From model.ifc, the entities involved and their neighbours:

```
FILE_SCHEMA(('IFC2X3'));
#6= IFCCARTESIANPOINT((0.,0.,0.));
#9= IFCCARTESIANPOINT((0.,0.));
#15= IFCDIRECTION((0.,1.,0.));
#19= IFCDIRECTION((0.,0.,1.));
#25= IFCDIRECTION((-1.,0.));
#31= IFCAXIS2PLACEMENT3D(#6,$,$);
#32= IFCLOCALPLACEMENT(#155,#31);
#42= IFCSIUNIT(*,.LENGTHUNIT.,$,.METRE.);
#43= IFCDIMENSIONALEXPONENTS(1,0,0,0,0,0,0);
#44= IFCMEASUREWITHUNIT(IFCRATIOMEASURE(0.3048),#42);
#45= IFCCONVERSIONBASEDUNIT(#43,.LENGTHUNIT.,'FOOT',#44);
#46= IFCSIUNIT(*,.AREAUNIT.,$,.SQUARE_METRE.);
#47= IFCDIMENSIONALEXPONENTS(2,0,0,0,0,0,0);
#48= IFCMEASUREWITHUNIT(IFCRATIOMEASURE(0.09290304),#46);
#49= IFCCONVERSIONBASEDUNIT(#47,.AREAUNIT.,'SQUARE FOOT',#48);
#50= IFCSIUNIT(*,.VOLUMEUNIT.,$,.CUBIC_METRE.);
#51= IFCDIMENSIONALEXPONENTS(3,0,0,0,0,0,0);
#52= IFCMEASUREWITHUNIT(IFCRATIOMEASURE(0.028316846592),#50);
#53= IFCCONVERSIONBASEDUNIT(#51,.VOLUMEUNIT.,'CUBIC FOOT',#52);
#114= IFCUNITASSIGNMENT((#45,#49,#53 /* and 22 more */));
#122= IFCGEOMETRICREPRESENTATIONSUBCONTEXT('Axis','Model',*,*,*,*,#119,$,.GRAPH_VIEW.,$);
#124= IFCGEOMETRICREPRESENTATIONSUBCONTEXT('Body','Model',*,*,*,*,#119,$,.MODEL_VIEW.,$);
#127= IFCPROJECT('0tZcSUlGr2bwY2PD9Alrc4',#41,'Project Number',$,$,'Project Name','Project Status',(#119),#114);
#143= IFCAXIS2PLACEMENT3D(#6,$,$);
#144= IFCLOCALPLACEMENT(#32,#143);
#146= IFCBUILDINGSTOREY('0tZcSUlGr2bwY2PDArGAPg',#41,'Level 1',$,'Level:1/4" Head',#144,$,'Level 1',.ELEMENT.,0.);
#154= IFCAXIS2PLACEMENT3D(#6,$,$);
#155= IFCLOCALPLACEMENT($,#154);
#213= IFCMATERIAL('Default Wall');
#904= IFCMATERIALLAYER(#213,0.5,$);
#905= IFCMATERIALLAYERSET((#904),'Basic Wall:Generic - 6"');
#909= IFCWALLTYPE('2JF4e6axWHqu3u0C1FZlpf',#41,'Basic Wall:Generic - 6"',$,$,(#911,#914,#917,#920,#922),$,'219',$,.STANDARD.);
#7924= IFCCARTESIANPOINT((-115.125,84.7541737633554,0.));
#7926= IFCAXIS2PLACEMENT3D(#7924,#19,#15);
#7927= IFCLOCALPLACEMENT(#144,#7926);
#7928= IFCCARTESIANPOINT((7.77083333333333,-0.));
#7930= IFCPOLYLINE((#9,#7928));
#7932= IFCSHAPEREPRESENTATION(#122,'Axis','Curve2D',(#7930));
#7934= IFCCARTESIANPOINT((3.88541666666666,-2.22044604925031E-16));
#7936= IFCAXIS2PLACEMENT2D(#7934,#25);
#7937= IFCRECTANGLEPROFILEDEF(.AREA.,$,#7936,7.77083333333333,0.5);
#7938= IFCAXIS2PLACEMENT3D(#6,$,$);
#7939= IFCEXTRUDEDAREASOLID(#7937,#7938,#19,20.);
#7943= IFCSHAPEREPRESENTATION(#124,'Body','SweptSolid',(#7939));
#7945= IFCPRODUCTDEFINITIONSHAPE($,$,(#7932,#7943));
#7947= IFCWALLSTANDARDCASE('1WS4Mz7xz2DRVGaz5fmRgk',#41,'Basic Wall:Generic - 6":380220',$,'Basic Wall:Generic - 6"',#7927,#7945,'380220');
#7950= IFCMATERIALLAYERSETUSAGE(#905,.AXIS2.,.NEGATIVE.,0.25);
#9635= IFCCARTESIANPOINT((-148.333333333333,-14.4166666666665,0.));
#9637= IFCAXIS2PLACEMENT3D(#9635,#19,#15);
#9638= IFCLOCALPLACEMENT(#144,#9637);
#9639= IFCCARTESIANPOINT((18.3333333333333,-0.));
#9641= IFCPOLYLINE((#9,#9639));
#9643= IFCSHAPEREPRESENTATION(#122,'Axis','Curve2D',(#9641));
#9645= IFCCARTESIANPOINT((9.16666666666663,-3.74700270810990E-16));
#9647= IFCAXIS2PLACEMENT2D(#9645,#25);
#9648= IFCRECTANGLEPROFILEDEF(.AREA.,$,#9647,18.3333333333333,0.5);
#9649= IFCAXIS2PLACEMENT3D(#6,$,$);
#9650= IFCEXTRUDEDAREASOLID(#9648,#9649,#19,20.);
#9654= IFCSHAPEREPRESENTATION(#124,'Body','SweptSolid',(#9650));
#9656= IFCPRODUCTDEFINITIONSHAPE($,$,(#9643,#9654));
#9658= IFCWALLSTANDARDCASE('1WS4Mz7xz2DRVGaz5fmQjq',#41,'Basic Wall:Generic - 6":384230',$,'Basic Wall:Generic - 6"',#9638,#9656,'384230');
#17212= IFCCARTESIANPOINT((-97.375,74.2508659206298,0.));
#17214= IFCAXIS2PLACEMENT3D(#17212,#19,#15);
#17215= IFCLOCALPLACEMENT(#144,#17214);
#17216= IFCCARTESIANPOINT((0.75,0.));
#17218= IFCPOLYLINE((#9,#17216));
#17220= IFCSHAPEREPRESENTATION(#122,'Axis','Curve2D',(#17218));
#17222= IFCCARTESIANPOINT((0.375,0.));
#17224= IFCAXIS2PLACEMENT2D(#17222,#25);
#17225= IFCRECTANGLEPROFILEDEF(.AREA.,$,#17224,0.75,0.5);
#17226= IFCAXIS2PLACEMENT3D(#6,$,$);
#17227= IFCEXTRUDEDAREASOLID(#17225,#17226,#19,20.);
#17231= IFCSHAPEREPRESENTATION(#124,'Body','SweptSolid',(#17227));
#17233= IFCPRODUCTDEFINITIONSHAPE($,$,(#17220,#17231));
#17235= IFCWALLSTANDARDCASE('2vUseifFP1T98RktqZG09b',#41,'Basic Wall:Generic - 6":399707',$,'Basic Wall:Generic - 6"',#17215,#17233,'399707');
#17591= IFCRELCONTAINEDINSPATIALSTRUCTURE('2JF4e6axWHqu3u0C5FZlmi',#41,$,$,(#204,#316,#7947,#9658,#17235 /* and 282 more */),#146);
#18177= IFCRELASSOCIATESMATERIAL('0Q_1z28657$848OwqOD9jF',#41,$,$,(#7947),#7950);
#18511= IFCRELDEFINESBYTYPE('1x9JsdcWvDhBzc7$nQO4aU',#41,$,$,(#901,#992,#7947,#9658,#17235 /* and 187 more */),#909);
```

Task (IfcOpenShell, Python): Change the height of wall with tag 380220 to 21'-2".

```python
import ifcopenshell
import ifcopenshell.geom
import ifcopenshell.util.representation
import ifcopenshell.util.shape
import ifcopenshell.util.unit

model = ifcopenshell.open("model.ifc")
unit_scale = ifcopenshell.util.unit.calculate_unit_scale(model)
settings = ifcopenshell.geom.settings()


def volume(element):
    """Net volume in cubic metres, openings subtracted."""
    shape = ifcopenshell.geom.create_shape(settings, element)
    return ifcopenshell.util.shape.get_volume(shape.geometry)


wall = model.by_guid("1WS4Mz7xz2DRVGaz5fmRgk")
before = volume(wall)

body = ifcopenshell.util.representation.get_representation(wall, "Model", "Body")
solid = body.Items[0]
old_height = solid.Depth
solid.Depth = 254 * 0.0254 / unit_scale
after = volume(wall)

print(f"height {old_height:g} -> {solid.Depth:g}, volume {before:.3f} -> {after:.3f} m3")

model.write("model_v2.ifc")
```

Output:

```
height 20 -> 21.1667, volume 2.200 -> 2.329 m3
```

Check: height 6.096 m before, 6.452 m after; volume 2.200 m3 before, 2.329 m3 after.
